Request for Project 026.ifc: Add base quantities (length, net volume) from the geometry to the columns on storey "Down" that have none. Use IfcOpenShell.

First a look at what the model holds.

```python
import ifcopenshell
import ifcopenshell.util.element
import ifcopenshell.util.unit

model = ifcopenshell.open("Project 026.ifc")
print(model.schema)
for unit_type in ("LENGTHUNIT", "AREAUNIT", "VOLUMEUNIT"):
    print(unit_type, ifcopenshell.util.unit.calculate_unit_scale(model, unit_type))
storey = next(s for s in model.by_type("IfcBuildingStorey") if s.Name == "Down")
columns = [e for e in ifcopenshell.util.element.get_decomposition(storey) if e.is_a("IfcColumn")]
for e in sorted(columns, key=lambda e: e.id()):
    print(e.id(), e.is_a(), e.Name, list(ifcopenshell.util.element.get_psets(e, qtos_only=True)), sep=" | ")
```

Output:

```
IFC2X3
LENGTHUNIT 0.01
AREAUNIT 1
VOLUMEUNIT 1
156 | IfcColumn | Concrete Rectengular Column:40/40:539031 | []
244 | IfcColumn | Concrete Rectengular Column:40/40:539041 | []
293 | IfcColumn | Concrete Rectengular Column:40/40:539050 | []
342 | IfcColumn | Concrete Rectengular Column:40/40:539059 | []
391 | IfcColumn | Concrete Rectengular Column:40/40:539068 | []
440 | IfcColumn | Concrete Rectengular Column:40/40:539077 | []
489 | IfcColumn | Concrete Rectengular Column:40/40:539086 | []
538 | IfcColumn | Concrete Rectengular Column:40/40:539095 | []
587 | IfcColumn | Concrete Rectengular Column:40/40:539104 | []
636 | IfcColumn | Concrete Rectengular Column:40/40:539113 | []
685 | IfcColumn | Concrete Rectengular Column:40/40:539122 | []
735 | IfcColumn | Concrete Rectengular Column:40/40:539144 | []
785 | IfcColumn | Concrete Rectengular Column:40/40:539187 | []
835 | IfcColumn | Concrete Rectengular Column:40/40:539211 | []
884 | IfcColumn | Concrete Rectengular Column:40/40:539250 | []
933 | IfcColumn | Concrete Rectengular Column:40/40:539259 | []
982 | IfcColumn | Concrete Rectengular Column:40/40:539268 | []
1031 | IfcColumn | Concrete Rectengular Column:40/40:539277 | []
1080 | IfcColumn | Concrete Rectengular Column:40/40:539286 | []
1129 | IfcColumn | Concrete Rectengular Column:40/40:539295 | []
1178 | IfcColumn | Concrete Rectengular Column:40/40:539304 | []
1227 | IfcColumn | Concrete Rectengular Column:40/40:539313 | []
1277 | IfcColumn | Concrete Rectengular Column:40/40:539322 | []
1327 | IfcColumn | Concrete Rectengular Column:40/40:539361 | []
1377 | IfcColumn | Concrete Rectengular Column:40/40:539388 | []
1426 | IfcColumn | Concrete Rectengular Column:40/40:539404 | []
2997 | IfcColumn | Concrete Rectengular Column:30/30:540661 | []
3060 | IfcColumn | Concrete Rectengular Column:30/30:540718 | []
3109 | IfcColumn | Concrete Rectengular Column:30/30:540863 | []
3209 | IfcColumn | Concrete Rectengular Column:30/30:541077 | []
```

```python
import ifcopenshell
import ifcopenshell.api.pset
import ifcopenshell.geom
import ifcopenshell.util.element
import ifcopenshell.util.shape
import ifcopenshell.util.unit

model = ifcopenshell.open("Project 026.ifc")
unit_scale = ifcopenshell.util.unit.calculate_unit_scale(model)
volume_scale = ifcopenshell.util.unit.calculate_unit_scale(model, "VOLUMEUNIT")
settings = ifcopenshell.geom.settings()

storey = next(s for s in model.by_type("IfcBuildingStorey") if s.Name == "Down")
columns = [e for e in ifcopenshell.util.element.get_decomposition(storey) if e.is_a("IfcColumn")]

for e in sorted(columns, key=lambda e: e.id()):
    if ifcopenshell.util.element.get_psets(e, qtos_only=True, should_inherit=False):
        continue
    # Geometry comes back in metres, in the element's own axes.
    shape = ifcopenshell.geom.create_shape(settings, e)
    values = {
        "Length": ifcopenshell.util.shape.get_z(shape.geometry) / unit_scale,
        "NetVolume": ifcopenshell.util.shape.get_volume(shape.geometry) / volume_scale,
    }
    qto = ifcopenshell.api.pset.add_qto(model, product=e, name="BaseQuantities")
    ifcopenshell.api.pset.edit_qto(model, qto=qto, properties=values)
    print(e.id(), {k: round(v, 3) for k, v in values.items()})

model.write("Project 026_rev.ifc")
```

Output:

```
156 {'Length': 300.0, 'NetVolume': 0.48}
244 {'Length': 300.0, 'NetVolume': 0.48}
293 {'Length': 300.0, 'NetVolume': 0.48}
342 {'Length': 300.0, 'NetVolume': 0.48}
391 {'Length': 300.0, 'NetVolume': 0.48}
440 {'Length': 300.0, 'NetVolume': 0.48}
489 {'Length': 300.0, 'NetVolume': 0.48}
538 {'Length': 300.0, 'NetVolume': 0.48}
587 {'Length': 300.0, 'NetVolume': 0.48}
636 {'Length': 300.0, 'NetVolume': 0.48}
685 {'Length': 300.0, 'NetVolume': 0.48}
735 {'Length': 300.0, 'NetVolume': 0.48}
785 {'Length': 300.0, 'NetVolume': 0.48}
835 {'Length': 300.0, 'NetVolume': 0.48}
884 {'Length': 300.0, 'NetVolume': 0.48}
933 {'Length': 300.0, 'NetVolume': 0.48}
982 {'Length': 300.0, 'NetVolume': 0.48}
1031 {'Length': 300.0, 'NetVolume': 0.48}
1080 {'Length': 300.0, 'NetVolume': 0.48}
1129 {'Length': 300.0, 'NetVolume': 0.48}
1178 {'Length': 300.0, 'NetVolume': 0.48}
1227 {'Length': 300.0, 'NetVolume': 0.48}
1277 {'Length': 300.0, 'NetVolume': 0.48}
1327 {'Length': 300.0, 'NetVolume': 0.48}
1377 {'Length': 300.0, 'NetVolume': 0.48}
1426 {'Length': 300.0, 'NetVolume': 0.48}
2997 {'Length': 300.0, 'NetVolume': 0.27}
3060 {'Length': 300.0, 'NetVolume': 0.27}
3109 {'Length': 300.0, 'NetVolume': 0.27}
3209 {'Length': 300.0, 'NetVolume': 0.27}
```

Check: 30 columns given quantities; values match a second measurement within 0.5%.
